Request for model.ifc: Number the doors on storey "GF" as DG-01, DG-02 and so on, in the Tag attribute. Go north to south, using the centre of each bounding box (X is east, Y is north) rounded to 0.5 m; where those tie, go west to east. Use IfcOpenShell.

First a look at what the model holds.

```python
import ifcopenshell
import ifcopenshell.util.element
import ifcopenshell.util.placement

model = ifcopenshell.open("model.ifc")
print(model.schema)
storey = next(s for s in model.by_type("IfcBuildingStorey") if s.Name == "GF")
doors = [e for e in ifcopenshell.util.element.get_decomposition(storey) if e.is_a("IfcDoor")]
for e in sorted(doors, key=lambda e: e.id()):
    origin = ifcopenshell.util.placement.get_local_placement(e.ObjectPlacement)[:3, 3]
    print(e.id(), e.Tag, e.Name, origin.round(2) + 0.0, sep=" | ")
```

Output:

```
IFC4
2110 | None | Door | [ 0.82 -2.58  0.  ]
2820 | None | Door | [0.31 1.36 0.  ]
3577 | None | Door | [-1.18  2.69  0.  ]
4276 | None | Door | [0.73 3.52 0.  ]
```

```python
import ifcopenshell
import ifcopenshell.geom
import ifcopenshell.util.element
import ifcopenshell.util.shape

model = ifcopenshell.open("model.ifc")
settings = ifcopenshell.geom.settings()
settings.set("use-world-coords", True)


def centre(element):
    shape = ifcopenshell.geom.create_shape(settings, element)
    return ifcopenshell.util.shape.get_bbox_centroid(shape.geometry)


storey = next(s for s in model.by_type("IfcBuildingStorey") if s.Name == "GF")
doors = [e for e in ifcopenshell.util.element.get_decomposition(storey) if e.is_a("IfcDoor")]

# Insertion points can sit at a corner or the storey origin, so sort by the geometry (in metres).
centres = {e: centre(e) for e in doors}
doors.sort(key=lambda e: (-round(centres[e][1] / 0.5), centres[e][0]))

for i, e in enumerate(doors, start=1):
    number = f"DG-{i:02d}"
    e.Tag = number
    print(e.id(), number)

model.write("model-out.ifc")
```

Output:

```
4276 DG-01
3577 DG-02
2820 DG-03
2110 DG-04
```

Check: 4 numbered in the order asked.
